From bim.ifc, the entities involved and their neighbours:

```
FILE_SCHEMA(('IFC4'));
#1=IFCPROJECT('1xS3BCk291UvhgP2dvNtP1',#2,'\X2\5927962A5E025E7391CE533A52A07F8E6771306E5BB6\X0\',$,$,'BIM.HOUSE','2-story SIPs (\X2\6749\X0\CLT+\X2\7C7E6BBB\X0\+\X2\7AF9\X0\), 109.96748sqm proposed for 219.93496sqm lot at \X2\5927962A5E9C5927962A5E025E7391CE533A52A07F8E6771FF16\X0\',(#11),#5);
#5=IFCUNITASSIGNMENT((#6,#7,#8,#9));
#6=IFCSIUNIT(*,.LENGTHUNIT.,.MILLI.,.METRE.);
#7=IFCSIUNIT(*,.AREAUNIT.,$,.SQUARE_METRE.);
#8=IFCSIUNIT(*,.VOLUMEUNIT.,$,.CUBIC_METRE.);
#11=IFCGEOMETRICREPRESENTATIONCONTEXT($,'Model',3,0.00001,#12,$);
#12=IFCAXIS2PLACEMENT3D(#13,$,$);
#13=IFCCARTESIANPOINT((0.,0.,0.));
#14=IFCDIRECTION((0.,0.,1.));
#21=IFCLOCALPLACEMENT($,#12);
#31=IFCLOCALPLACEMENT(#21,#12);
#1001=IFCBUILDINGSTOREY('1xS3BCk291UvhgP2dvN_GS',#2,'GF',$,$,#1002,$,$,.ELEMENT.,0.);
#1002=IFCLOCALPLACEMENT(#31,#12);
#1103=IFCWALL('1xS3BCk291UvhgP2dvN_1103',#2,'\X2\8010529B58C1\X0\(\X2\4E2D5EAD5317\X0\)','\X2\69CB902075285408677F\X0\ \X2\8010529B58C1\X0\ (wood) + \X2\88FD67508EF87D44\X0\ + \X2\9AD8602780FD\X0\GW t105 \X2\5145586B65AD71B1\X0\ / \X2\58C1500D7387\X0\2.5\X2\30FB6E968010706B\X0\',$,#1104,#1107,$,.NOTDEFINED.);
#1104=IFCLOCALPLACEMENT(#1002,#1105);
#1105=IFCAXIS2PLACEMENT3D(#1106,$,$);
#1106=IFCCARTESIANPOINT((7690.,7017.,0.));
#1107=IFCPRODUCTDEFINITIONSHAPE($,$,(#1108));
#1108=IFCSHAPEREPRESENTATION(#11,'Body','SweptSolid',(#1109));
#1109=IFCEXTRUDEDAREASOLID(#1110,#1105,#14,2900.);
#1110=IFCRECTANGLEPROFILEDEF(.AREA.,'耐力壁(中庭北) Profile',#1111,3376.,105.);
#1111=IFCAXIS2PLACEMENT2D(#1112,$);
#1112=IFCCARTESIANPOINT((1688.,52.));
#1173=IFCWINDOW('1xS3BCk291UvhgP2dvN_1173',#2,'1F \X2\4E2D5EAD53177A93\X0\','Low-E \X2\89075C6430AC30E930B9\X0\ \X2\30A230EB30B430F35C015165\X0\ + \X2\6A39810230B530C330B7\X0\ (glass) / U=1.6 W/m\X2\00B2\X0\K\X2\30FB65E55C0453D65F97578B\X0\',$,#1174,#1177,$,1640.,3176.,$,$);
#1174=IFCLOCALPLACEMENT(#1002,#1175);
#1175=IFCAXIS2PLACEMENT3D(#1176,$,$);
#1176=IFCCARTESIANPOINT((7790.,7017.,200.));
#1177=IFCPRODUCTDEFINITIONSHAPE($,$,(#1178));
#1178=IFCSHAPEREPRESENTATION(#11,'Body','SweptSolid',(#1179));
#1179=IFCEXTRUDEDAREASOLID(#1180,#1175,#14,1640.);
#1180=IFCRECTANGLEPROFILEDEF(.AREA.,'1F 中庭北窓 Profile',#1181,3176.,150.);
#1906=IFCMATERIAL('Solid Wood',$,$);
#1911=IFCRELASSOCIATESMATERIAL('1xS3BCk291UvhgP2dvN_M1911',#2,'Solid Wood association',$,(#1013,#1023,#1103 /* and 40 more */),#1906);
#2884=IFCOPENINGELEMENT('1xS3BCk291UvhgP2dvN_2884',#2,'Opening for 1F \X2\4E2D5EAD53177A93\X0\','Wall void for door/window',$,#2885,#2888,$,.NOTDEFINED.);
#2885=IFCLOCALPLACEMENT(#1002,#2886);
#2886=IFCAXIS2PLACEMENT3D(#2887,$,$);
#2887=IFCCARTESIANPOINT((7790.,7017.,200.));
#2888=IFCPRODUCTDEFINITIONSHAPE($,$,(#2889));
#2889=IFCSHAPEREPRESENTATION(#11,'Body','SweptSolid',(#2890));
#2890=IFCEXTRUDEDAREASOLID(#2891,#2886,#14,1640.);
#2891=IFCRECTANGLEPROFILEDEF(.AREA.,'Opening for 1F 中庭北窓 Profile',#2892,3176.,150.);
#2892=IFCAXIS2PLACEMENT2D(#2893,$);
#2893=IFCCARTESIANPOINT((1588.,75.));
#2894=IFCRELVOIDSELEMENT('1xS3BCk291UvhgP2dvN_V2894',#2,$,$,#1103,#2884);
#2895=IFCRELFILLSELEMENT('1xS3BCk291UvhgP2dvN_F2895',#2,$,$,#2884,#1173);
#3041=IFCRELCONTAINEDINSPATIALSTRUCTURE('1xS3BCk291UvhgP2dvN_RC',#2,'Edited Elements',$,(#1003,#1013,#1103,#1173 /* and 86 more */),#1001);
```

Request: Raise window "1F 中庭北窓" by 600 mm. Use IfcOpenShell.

```python
import numpy as np
import ifcopenshell
import ifcopenshell.api.geometry
import ifcopenshell.util.placement
import ifcopenshell.util.unit

model = ifcopenshell.open("bim.ifc")
unit_scale = ifcopenshell.util.unit.calculate_unit_scale(model)

window = model.by_guid("1xS3BCk291UvhgP2dvN_1173")
opening = window.FillsVoids[0].RelatingOpeningElement
dz = 0.6 / unit_scale

shift = np.array([0.0, 0.0, dz])
# The window is not placed relative to its opening, so move both.
for product in (opening, window):
    matrix = ifcopenshell.util.placement.get_local_placement(product.ObjectPlacement)
    matrix[:3, 3] += shift
    ifcopenshell.api.geometry.edit_object_placement(model, product=product, matrix=matrix, is_si=False)

print(f"moved by {dz * unit_scale:+.3f} m")

model.write("bim_updated.ifc")
```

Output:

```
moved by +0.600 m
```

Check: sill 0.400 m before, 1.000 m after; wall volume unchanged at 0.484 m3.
